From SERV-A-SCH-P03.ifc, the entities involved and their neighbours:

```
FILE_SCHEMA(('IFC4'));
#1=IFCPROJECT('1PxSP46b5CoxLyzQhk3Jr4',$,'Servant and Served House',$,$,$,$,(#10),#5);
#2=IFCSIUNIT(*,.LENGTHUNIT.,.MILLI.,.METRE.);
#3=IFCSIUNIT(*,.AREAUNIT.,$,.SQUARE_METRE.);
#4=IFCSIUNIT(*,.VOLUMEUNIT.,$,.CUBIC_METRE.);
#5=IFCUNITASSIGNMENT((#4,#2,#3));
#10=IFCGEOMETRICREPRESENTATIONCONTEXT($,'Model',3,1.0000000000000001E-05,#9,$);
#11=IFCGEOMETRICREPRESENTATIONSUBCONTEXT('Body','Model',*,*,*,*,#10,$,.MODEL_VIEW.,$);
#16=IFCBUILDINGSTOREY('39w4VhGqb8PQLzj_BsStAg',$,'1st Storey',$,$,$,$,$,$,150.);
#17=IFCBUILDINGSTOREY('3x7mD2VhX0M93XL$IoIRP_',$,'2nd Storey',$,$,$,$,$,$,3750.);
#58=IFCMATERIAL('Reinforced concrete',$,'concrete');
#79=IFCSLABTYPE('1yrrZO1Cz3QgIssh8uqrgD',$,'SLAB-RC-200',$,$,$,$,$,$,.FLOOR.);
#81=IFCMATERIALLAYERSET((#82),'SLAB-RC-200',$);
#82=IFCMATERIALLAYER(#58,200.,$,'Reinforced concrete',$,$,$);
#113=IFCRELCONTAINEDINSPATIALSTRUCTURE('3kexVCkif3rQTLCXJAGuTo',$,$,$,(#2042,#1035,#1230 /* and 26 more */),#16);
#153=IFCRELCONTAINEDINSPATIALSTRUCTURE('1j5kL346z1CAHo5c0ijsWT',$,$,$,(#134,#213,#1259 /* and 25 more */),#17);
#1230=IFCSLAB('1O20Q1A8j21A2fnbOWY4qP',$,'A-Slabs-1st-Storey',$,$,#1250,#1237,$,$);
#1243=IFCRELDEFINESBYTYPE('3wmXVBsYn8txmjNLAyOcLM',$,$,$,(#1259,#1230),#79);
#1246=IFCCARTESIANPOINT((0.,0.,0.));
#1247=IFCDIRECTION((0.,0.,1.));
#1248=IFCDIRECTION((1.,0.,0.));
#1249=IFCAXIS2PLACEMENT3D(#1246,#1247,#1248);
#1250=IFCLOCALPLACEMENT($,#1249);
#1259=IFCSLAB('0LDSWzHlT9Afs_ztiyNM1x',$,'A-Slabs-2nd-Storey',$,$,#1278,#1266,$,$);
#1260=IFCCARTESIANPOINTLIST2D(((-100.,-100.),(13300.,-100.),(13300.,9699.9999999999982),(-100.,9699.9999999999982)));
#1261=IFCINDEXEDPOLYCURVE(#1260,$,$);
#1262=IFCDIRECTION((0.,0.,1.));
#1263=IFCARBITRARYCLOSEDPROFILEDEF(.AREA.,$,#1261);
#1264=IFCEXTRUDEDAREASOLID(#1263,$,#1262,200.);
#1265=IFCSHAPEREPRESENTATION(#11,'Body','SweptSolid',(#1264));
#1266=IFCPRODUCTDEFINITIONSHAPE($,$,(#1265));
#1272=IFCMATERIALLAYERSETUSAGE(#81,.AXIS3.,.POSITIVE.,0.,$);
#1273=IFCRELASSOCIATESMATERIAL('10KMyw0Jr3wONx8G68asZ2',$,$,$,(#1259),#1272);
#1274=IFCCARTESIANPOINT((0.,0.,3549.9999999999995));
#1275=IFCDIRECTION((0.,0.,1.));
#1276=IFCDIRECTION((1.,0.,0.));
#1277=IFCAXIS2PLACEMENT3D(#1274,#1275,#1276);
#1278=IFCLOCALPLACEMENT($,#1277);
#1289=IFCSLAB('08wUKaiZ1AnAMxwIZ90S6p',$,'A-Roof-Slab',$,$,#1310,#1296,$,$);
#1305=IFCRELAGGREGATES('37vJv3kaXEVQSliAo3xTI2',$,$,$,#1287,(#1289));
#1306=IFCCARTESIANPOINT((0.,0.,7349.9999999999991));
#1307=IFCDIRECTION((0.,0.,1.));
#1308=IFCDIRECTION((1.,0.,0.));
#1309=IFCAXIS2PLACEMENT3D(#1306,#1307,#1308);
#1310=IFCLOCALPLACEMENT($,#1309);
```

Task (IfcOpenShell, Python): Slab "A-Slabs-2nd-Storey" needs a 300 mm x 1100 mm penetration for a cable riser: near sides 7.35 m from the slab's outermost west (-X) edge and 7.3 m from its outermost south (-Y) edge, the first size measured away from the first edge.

```python
import numpy as np
import ifcopenshell
import ifcopenshell.api.feature
import ifcopenshell.api.geometry
import ifcopenshell.api.root
import ifcopenshell.geom
import ifcopenshell.util.placement
import ifcopenshell.util.representation
import ifcopenshell.util.shape
import ifcopenshell.util.unit

model = ifcopenshell.open("SERV-A-SCH-P03.ifc")
unit_scale = ifcopenshell.util.unit.calculate_unit_scale(model)
settings = ifcopenshell.geom.settings()


def volume(element):
    """Net volume in cubic metres, openings subtracted."""
    shape = ifcopenshell.geom.create_shape(settings, element)
    return ifcopenshell.util.shape.get_volume(shape.geometry)


slab = model.by_guid("0LDSWzHlT9Afs_ztiyNM1x")
before = volume(slab)

# Extent in the slab's own axes, in metres. The edges named are its -X and -Y sides.
slab_shape = ifcopenshell.geom.create_shape(settings, slab)
vertices = ifcopenshell.util.shape.get_vertices(slab_shape.geometry)
x_min, y_min, bottom = vertices.min(axis=0)
top = vertices[:, 2].max()

opening = ifcopenshell.api.root.create_entity(model, ifc_class="IfcOpeningElement", name="Cable riser opening", predefined_type="OPENING")
context = ifcopenshell.util.representation.get_context(model, "Model", "Body", "MODEL_VIEW")
width, depth = 0.3, 1.1
outline = [(0.0, 0.0), (width, 0.0), (width, depth), (0.0, depth), (0.0, 0.0)]
# Overshoot both faces by 50 mm so the cut is clean.
shape = ifcopenshell.api.geometry.add_slab_representation(
    model, context=context, depth=top - bottom + 0.1, polyline=outline
)
ifcopenshell.api.geometry.assign_representation(model, product=opening, representation=shape)

matrix = ifcopenshell.util.placement.get_local_placement(slab.ObjectPlacement)
matrix[:, 3] = matrix @ np.append(np.array([x_min + 7.35, y_min + 7.3, bottom - 0.05]) / unit_scale, 1.0)
ifcopenshell.api.geometry.edit_object_placement(model, product=opening, matrix=matrix, is_si=False)
ifcopenshell.api.feature.add_feature(model, feature=opening, element=slab)

after = volume(slab)

print(f"slab volume {before:.3f} -> {after:.3f} m3")

model.write("SERV-A-SCH-P03_v2.ifc")
```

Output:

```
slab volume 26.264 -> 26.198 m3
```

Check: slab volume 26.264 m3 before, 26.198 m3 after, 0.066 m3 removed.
